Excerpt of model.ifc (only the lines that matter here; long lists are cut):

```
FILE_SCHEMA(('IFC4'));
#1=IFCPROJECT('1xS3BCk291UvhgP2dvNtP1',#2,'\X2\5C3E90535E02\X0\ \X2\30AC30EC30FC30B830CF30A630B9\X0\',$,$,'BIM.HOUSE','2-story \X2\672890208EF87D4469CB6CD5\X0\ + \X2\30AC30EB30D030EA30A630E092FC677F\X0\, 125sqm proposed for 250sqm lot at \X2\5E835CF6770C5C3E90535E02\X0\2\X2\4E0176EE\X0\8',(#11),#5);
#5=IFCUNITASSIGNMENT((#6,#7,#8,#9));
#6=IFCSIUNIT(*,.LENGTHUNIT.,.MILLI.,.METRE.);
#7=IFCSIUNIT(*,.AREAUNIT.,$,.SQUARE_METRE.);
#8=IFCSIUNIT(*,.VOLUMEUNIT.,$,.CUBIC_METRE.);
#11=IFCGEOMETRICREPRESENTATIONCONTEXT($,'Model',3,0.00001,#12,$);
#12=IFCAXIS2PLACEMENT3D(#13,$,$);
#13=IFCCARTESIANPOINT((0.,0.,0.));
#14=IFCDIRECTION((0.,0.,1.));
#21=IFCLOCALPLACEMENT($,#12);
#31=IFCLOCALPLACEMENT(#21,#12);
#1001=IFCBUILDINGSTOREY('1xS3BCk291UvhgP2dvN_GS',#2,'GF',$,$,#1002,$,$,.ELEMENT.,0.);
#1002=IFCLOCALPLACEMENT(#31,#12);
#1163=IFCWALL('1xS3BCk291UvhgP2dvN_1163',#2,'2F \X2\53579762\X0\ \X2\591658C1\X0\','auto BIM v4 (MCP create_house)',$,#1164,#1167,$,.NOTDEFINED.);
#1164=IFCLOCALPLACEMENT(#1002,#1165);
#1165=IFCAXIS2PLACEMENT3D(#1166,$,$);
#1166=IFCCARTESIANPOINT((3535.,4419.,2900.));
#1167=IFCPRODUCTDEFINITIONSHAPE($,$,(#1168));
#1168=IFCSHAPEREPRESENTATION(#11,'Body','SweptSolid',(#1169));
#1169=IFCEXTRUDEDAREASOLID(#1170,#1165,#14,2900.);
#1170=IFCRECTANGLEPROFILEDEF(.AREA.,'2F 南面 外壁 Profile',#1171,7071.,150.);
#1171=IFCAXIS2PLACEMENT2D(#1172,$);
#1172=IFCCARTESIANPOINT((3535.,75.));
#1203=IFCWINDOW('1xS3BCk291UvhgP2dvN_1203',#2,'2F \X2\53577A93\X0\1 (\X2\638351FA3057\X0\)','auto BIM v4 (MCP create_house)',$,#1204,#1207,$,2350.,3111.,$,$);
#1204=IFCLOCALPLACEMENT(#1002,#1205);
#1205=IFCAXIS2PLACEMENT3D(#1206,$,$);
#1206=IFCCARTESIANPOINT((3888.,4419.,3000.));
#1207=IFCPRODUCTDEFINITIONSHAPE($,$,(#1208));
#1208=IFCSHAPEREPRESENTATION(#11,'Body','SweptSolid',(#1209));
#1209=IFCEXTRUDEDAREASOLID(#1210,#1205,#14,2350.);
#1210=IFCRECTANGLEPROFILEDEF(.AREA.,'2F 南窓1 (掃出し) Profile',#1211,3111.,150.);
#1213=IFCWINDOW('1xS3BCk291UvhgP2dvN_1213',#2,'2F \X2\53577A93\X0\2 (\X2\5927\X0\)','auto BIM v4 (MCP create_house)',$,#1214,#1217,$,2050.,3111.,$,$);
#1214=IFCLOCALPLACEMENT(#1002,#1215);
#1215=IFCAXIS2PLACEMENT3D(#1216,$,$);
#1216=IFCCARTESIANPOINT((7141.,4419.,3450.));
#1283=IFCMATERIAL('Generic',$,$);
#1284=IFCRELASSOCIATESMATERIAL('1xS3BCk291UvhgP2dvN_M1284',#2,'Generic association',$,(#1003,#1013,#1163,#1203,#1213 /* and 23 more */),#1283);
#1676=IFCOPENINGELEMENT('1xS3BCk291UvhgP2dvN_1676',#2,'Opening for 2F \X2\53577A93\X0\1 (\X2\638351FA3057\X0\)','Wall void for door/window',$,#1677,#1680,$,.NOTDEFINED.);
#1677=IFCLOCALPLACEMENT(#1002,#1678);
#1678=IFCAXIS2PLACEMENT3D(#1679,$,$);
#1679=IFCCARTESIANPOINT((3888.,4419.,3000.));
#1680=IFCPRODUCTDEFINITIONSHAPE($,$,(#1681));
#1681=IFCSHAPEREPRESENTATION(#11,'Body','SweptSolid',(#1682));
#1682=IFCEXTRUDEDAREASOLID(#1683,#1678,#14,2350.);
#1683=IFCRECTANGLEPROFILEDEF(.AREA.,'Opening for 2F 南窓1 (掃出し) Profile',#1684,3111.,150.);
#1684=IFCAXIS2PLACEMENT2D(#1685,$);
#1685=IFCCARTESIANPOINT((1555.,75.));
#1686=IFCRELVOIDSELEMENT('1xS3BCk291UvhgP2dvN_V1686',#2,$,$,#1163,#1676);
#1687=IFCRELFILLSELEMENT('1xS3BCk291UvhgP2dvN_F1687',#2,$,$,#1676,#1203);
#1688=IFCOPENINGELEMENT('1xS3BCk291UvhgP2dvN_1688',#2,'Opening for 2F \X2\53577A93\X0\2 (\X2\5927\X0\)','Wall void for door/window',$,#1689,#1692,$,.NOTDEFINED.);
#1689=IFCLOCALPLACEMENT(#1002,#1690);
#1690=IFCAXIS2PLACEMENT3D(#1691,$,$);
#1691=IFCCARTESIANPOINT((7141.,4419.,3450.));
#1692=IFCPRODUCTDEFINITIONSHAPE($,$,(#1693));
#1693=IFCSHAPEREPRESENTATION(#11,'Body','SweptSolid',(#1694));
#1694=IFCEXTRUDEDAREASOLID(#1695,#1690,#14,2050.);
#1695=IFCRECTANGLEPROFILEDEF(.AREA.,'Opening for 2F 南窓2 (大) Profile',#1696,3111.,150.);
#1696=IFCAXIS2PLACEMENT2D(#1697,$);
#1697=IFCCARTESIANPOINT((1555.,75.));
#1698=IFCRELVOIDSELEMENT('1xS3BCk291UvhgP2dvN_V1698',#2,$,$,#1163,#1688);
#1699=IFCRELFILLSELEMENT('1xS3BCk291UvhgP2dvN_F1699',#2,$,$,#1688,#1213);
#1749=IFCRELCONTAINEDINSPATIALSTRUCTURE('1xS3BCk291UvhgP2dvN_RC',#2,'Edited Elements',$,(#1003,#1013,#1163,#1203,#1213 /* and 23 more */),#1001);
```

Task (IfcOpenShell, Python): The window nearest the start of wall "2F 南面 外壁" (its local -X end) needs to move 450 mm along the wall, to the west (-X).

```python
import ifcopenshell
import ifcopenshell.api.geometry
import ifcopenshell.util.placement

model = ifcopenshell.open("model.ifc")

window = model.by_id(1203)
opening = window.FillsVoids[0].RelatingOpeningElement
wall = opening.VoidsElements[0].RelatingBuildingElement

wall_matrix = ifcopenshell.util.placement.get_local_placement(wall.ObjectPlacement)
shift = wall_matrix[:3, 0] * -450.0
before = ifcopenshell.util.placement.get_local_placement(window.ObjectPlacement)[:3, 3].copy()

# The window is not placed relative to its opening, so move both.
for product in (opening, window):
    matrix = ifcopenshell.util.placement.get_local_placement(product.ObjectPlacement)
    matrix[:3, 3] += shift
    ifcopenshell.api.geometry.edit_object_placement(model, product=product, matrix=matrix, is_si=False)

after = ifcopenshell.util.placement.get_local_placement(window.ObjectPlacement)[:3, 3]
print("window moved by", (after - before).round(3) + 0.0)

model.write("model_rev.ifc")
```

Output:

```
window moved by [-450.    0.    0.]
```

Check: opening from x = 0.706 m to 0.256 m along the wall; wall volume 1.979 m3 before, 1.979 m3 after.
